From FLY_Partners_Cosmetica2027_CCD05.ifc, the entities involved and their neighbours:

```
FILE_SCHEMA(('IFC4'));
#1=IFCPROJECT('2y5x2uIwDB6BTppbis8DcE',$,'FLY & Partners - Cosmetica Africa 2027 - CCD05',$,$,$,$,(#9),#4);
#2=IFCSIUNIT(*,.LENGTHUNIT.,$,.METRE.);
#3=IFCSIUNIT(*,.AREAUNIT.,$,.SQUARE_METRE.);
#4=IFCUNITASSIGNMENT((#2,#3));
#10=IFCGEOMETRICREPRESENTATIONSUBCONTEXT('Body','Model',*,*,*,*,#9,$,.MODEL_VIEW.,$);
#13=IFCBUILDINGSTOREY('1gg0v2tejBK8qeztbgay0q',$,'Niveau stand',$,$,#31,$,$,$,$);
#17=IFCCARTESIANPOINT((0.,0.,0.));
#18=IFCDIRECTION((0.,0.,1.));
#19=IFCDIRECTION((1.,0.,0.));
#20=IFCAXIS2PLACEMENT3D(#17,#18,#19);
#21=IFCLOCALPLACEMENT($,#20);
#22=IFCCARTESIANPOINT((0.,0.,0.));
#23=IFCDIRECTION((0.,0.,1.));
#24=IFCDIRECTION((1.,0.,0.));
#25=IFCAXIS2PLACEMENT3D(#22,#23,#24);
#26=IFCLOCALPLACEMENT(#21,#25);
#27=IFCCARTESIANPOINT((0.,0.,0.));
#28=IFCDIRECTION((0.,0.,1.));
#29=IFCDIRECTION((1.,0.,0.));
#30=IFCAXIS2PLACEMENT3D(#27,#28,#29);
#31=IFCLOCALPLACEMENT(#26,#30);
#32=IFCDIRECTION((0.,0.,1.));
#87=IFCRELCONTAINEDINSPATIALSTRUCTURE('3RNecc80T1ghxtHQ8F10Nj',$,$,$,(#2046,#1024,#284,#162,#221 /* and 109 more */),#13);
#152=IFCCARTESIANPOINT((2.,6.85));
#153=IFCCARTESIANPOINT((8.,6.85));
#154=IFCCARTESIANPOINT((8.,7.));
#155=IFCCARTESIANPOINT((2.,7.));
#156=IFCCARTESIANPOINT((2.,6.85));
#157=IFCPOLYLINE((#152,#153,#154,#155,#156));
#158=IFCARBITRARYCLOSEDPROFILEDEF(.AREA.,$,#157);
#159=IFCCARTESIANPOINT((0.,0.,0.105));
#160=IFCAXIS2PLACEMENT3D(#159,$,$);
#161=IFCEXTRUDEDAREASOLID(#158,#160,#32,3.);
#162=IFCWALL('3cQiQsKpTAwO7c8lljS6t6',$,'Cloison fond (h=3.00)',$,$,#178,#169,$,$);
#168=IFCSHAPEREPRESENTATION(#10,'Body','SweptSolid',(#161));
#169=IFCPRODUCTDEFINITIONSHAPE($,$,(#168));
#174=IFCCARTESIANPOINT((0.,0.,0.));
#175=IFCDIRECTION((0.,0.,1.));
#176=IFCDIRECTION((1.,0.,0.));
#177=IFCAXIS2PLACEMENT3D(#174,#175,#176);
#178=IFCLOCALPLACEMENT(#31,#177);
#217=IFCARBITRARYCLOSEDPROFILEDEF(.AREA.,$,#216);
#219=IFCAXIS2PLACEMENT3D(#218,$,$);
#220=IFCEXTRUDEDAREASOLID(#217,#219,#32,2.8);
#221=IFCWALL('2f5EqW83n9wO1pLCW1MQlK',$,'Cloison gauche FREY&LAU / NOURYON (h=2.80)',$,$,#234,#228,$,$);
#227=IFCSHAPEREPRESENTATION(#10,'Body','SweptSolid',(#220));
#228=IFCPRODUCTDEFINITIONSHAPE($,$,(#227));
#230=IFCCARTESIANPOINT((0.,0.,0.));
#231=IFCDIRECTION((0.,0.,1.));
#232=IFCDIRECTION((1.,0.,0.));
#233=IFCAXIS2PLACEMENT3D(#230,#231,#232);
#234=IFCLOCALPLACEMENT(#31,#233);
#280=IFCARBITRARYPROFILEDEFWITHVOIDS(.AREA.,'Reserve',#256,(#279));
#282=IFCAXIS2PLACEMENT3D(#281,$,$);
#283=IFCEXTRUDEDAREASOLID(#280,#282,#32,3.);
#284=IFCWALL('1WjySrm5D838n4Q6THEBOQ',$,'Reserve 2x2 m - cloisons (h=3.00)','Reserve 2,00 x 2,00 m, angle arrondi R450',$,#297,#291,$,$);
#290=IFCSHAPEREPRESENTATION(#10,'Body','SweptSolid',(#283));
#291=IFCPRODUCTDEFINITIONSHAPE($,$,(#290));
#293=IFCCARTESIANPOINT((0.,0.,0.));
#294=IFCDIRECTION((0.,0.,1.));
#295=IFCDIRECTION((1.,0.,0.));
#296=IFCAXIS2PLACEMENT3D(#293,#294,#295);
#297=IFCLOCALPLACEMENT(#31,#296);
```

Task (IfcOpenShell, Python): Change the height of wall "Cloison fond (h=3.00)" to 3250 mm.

```python
import ifcopenshell
import ifcopenshell.geom
import ifcopenshell.util.representation
import ifcopenshell.util.shape
import ifcopenshell.util.unit

model = ifcopenshell.open("FLY_Partners_Cosmetica2027_CCD05.ifc")
unit_scale = ifcopenshell.util.unit.calculate_unit_scale(model)
settings = ifcopenshell.geom.settings()


def volume(element):
    """Net volume in cubic metres, openings subtracted."""
    shape = ifcopenshell.geom.create_shape(settings, element)
    return ifcopenshell.util.shape.get_volume(shape.geometry)


wall = model.by_guid("3cQiQsKpTAwO7c8lljS6t6")
before = volume(wall)

body = ifcopenshell.util.representation.get_representation(wall, "Model", "Body")
solid = body.Items[0]
old_height = solid.Depth
solid.Depth = 3.25 / unit_scale
after = volume(wall)

print(f"height {old_height:g} -> {solid.Depth:g}, volume {before:.3f} -> {after:.3f} m3")

model.write("FLY_Partners_Cosmetica2027_CCD05_edited.ifc")
```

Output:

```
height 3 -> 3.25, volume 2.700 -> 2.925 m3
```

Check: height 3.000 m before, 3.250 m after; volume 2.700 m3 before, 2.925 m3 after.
